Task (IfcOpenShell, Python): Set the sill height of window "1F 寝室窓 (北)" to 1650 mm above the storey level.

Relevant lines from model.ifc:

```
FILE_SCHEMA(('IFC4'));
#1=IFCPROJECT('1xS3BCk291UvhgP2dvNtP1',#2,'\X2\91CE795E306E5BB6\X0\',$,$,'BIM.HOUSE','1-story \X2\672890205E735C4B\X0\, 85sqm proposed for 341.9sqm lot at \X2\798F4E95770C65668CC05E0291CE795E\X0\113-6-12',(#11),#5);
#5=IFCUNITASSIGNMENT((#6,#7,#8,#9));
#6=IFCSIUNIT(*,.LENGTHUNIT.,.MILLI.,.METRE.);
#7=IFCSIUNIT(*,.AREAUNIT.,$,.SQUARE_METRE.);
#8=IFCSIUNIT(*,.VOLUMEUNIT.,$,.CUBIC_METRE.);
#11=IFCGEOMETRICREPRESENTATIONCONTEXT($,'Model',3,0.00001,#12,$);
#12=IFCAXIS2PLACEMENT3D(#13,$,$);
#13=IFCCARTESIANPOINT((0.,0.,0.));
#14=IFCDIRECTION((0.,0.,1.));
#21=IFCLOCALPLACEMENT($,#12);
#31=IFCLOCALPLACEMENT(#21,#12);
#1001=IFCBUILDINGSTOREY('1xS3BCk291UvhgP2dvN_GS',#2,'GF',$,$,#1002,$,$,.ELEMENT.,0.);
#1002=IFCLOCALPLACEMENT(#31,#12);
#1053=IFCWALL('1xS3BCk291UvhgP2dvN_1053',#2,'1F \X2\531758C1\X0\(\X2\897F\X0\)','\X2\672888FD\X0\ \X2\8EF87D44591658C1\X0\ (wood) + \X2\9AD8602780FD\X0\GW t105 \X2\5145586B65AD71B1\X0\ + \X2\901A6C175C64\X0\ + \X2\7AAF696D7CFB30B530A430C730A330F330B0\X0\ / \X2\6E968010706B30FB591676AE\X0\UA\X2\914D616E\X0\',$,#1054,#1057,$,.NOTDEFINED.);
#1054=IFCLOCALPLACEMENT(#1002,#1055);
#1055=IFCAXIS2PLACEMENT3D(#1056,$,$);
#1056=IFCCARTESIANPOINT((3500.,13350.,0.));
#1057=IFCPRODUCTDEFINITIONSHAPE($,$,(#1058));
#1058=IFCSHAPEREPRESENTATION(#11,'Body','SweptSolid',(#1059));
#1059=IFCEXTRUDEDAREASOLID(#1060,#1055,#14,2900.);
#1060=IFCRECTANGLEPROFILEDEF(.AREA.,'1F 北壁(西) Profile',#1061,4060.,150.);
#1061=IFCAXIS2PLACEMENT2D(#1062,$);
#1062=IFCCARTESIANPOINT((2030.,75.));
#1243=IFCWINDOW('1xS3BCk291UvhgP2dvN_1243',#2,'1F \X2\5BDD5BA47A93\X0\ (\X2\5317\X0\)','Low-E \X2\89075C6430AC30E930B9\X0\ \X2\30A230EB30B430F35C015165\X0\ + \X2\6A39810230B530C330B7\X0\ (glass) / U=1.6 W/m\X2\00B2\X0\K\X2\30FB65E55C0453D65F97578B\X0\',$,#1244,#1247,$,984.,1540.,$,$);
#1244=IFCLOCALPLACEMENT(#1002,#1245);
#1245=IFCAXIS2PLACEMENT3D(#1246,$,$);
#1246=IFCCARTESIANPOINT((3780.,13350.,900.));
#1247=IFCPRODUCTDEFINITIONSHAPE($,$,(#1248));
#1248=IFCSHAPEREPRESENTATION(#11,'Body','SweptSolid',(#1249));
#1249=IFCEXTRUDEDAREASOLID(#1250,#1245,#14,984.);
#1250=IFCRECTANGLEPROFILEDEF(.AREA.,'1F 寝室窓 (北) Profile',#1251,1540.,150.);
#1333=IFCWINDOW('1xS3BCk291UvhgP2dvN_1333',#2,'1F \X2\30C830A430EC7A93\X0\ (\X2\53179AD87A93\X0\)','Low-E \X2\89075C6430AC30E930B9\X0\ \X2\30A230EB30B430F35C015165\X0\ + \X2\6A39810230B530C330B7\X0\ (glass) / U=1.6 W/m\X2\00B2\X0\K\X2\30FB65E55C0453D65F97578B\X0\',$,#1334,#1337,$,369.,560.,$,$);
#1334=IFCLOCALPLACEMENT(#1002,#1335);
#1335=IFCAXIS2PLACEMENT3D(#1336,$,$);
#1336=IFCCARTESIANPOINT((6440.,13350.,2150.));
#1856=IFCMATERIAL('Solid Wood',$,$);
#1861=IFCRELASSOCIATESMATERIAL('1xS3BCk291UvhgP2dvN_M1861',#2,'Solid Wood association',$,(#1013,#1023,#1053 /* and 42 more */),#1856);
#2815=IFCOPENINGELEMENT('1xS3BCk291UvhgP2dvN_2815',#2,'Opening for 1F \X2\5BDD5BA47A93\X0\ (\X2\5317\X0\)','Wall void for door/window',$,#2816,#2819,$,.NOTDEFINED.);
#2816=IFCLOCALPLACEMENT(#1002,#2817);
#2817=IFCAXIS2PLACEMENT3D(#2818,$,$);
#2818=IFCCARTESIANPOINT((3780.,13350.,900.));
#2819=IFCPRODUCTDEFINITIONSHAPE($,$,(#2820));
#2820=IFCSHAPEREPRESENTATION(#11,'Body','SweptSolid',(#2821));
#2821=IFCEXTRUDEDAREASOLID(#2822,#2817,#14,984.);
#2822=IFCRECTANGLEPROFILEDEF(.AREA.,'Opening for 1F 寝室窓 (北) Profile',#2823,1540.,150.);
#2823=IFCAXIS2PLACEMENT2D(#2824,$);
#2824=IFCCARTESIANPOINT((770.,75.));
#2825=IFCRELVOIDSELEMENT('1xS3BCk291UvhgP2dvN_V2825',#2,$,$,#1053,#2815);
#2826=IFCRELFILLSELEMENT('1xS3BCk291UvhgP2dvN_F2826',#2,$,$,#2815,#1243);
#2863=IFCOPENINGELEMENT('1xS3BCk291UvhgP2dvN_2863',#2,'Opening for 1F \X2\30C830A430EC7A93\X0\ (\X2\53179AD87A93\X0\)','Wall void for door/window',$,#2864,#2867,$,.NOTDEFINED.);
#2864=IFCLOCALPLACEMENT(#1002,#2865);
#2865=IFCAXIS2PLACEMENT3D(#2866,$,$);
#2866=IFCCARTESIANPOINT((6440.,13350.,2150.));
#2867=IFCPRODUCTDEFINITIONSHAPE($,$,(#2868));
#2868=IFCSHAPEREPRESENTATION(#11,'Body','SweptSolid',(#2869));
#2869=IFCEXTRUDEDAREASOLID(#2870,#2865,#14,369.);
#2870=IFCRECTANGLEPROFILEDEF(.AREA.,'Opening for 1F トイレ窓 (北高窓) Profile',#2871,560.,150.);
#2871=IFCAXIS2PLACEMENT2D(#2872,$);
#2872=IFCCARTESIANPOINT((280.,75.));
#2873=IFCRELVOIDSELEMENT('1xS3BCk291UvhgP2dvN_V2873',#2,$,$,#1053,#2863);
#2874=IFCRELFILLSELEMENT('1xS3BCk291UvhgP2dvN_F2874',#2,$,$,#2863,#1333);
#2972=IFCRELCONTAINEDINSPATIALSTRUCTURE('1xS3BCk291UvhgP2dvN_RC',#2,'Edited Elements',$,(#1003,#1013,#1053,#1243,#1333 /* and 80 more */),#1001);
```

```python
import numpy as np
import ifcopenshell
import ifcopenshell.api.geometry
import ifcopenshell.geom
import ifcopenshell.util.element
import ifcopenshell.util.placement
import ifcopenshell.util.shape
import ifcopenshell.util.unit

model = ifcopenshell.open("model.ifc")
unit_scale = ifcopenshell.util.unit.calculate_unit_scale(model)

window = model.by_guid("1xS3BCk291UvhgP2dvN_1243")
opening = window.FillsVoids[0].RelatingOpeningElement
storey = ifcopenshell.util.element.get_container(window, ifc_class="IfcBuildingStorey")
level = ifcopenshell.util.placement.get_local_placement(storey.ObjectPlacement)[2, 3]

# The opening's origin need not be at the sill, so measure its lowest point.
shape = ifcopenshell.geom.create_shape(ifcopenshell.geom.settings(), opening)
bottom = ifcopenshell.util.shape.get_shape_bottom_elevation(shape, shape.geometry) / unit_scale
dz = level + 1650.0 - bottom

shift = np.array([0.0, 0.0, dz])
# The window is not placed relative to its opening, so move both.
for product in (opening, window):
    matrix = ifcopenshell.util.placement.get_local_placement(product.ObjectPlacement)
    matrix[:3, 3] += shift
    ifcopenshell.api.geometry.edit_object_placement(model, product=product, matrix=matrix, is_si=False)

print(f"moved by {dz * unit_scale:+.3f} m")

model.write("model_v2.ifc")
```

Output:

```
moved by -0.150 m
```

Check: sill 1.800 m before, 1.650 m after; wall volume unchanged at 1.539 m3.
